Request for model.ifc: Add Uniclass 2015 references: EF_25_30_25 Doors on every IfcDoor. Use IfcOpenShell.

First a look at what the model holds.

```python
import ifcopenshell

model = ifcopenshell.open("model.ifc")
print(model.schema)
print("classifications:", [c.Name for c in model.by_type("IfcClassification")])
for ifc_class in ("IfcDoor", "IfcRoof", "IfcStair", "IfcWall", "IfcWindow"):
    print(ifc_class, len(model.by_type(ifc_class)))
```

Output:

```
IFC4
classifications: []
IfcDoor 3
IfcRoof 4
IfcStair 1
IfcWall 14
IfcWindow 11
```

```python
import ifcopenshell
import ifcopenshell.api.classification

model = ifcopenshell.open("model.ifc")

system = ifcopenshell.api.classification.add_classification(model, classification="Uniclass 2015")

codes = {
    "IfcDoor": ("EF_25_30_25", "Doors"),
}
for ifc_class, (code, name) in codes.items():
    products = model.by_type(ifc_class)
    ifcopenshell.api.classification.add_reference(
        model, products=products, classification=system, identification=code, name=name
    )
    print(code, len(products))

model.write("model_edited.ifc")
```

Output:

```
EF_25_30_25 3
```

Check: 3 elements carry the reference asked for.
